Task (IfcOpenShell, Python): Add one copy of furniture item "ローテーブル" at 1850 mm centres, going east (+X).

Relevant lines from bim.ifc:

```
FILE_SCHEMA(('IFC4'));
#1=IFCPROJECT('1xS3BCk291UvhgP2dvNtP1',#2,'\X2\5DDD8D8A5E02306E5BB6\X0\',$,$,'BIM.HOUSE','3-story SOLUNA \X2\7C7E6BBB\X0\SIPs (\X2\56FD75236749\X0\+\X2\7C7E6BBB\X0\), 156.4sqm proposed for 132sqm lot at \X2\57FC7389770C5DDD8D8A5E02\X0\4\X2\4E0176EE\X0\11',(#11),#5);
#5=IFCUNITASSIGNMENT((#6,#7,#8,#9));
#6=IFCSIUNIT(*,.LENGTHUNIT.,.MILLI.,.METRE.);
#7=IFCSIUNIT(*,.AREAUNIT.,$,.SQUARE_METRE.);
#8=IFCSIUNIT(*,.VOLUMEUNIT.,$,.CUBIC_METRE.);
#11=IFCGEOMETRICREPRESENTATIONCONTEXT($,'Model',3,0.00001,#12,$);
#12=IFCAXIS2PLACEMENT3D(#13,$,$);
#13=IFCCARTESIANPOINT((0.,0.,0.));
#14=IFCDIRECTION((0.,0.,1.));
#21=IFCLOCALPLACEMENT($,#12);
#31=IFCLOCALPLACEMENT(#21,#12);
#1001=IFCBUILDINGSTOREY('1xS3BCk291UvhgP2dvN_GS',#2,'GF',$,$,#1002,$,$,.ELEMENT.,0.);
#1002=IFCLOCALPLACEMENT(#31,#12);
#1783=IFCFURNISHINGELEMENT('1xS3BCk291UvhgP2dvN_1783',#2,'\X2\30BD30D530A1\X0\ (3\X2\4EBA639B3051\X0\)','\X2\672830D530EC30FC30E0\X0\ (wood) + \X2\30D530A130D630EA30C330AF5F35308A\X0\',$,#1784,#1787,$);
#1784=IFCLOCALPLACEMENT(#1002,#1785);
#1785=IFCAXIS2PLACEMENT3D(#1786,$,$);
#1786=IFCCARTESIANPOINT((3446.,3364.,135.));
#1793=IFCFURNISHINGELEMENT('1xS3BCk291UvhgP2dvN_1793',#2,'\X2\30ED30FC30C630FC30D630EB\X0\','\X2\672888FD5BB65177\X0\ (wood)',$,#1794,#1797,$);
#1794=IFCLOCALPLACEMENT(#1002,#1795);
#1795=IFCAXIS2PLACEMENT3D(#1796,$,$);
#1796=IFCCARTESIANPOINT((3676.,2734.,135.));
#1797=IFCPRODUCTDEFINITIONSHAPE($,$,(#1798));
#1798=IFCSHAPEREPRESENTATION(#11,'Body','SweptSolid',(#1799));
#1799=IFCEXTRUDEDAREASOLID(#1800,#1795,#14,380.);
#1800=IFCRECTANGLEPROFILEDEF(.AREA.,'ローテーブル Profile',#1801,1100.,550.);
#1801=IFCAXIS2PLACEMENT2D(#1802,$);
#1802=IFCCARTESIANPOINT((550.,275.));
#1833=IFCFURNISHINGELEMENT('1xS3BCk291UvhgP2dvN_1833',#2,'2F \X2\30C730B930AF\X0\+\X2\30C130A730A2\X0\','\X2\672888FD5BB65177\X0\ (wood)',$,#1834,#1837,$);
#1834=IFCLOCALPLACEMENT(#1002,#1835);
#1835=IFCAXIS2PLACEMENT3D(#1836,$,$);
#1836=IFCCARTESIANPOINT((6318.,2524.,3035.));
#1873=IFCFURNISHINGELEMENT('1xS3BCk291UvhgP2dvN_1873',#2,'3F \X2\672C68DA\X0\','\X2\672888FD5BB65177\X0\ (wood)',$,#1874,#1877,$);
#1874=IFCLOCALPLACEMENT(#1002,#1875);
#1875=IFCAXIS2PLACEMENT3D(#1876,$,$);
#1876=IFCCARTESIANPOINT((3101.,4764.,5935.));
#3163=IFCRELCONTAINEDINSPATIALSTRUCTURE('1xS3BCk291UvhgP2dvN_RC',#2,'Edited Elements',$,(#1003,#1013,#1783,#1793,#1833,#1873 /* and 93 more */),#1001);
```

```python
import numpy as np
import ifcopenshell
import ifcopenshell.api.geometry
import ifcopenshell.api.root
import ifcopenshell.util.element
import ifcopenshell.util.placement

model = ifcopenshell.open("bim.ifc")


def reuse_history(source, copy):
    """copy_class also copies each property set's owner history, people and application; keep the originals."""
    for rel in copy.IsDefinedBy:
        if rel.is_a("IfcRelDefinesByProperties") and (history := rel.RelatingPropertyDefinition.OwnerHistory):
            rel.RelatingPropertyDefinition.OwnerHistory = source.OwnerHistory
            ifcopenshell.util.element.remove_deep2(model, history)


source = model.by_guid("1xS3BCk291UvhgP2dvN_1793")
base = ifcopenshell.util.placement.get_local_placement(source.ObjectPlacement)
step = np.array([1.0, 0.0, 0.0]) * 1850.0

for i in range(1, 2):
    copy = ifcopenshell.api.root.copy_class(model, product=source)
    copy.Representation = ifcopenshell.util.element.copy_deep(
        model, source.Representation, exclude=["IfcGeometricRepresentationContext", "IfcRepresentationMap"]
    )
    reuse_history(source, copy)
    matrix = base.copy()
    matrix[:3, 3] += i * step
    print("added at", matrix[:3, 3].round(3) + 0.0)
    ifcopenshell.api.geometry.edit_object_placement(model, product=copy, matrix=matrix, is_si=False)

model.write("bim_updated.ifc")
```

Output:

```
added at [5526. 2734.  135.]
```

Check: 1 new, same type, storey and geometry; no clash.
